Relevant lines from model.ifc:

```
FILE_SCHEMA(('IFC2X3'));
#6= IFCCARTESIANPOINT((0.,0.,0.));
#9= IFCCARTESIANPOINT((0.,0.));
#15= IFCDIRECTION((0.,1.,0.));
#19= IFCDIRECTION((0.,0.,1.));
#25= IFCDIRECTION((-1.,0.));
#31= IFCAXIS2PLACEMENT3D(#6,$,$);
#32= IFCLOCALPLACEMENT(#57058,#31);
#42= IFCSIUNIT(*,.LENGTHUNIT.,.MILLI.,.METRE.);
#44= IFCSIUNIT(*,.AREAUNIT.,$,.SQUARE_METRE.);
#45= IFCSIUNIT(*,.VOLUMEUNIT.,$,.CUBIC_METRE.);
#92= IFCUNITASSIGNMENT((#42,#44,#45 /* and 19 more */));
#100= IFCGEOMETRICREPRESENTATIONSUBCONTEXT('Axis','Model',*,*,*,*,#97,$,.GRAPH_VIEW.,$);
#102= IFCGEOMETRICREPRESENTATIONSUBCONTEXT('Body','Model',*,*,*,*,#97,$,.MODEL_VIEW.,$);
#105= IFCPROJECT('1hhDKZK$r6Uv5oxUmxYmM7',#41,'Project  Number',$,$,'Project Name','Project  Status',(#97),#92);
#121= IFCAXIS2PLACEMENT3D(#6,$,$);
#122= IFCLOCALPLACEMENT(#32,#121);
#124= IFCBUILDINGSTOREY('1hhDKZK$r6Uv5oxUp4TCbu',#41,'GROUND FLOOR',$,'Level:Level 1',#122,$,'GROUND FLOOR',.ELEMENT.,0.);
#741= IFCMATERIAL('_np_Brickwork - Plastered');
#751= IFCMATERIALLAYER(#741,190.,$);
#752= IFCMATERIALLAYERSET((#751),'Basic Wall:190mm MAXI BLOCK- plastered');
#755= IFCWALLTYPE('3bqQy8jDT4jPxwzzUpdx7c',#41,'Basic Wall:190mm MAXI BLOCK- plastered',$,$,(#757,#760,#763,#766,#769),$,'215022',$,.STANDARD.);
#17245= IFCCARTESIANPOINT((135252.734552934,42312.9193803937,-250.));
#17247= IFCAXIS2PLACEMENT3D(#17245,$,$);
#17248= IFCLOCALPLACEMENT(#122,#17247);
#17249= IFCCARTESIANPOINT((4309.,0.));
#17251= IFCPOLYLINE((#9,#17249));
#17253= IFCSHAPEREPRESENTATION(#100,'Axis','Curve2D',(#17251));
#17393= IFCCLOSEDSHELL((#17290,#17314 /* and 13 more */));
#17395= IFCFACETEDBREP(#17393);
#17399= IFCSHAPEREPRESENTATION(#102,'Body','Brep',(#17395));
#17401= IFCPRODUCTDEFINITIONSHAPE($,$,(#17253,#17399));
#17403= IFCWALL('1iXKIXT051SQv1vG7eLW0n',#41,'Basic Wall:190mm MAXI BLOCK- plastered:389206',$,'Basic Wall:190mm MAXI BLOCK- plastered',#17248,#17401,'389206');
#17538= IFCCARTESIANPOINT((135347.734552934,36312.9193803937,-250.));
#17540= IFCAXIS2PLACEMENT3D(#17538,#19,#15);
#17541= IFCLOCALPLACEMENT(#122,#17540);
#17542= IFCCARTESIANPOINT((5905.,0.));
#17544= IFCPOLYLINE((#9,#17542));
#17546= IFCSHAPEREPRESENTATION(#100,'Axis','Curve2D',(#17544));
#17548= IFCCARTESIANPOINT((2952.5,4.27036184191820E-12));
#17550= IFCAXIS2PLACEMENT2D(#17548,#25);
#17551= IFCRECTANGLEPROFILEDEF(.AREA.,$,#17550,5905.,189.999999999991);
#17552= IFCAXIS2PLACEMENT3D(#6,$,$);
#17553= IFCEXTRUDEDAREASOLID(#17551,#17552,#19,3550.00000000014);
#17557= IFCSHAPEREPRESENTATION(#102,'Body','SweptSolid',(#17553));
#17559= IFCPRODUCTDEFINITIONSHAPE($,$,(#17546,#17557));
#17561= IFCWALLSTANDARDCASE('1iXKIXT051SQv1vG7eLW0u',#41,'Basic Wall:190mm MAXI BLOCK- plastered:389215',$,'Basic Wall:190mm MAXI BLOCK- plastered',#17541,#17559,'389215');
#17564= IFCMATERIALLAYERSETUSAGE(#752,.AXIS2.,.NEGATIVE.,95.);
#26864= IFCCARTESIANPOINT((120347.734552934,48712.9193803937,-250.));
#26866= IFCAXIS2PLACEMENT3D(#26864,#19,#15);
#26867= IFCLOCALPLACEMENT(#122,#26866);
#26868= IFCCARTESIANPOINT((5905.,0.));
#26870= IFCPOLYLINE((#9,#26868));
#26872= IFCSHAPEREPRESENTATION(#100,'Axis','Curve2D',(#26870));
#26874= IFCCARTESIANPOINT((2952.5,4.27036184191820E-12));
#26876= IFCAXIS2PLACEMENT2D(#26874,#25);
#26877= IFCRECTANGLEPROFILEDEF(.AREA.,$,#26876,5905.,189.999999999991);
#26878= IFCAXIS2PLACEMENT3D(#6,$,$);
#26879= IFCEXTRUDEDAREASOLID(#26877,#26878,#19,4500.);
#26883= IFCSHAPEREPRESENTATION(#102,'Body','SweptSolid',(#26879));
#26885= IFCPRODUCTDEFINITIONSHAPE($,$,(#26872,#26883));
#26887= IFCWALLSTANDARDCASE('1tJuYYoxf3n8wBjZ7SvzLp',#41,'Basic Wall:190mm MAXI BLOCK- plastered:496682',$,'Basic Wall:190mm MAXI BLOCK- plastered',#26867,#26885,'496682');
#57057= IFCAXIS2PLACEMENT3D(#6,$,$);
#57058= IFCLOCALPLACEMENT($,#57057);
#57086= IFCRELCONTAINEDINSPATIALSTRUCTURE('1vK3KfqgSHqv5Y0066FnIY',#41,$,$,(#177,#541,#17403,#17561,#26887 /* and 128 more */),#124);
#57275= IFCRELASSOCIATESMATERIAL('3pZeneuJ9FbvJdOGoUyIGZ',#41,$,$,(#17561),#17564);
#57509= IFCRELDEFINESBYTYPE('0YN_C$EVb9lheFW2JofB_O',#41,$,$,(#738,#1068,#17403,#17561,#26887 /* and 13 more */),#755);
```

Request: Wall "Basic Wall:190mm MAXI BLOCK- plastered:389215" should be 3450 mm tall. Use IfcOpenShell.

```python
import ifcopenshell
import ifcopenshell.geom
import ifcopenshell.util.representation
import ifcopenshell.util.shape
import ifcopenshell.util.unit

model = ifcopenshell.open("model.ifc")
unit_scale = ifcopenshell.util.unit.calculate_unit_scale(model)
settings = ifcopenshell.geom.settings()


def volume(element):
    """Net volume in cubic metres, openings subtracted."""
    shape = ifcopenshell.geom.create_shape(settings, element)
    return ifcopenshell.util.shape.get_volume(shape.geometry)


wall = model.by_id(17561)
before = volume(wall)

body = ifcopenshell.util.representation.get_representation(wall, "Model", "Body")
solid = body.Items[0]
old_height = solid.Depth
solid.Depth = 3.45 / unit_scale
after = volume(wall)

print(f"height {old_height:g} -> {solid.Depth:g}, volume {before:.3f} -> {after:.3f} m3")

model.write("model_v2.ifc")
```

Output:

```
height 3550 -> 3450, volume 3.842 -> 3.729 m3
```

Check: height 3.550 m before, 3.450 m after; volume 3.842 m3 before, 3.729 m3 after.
